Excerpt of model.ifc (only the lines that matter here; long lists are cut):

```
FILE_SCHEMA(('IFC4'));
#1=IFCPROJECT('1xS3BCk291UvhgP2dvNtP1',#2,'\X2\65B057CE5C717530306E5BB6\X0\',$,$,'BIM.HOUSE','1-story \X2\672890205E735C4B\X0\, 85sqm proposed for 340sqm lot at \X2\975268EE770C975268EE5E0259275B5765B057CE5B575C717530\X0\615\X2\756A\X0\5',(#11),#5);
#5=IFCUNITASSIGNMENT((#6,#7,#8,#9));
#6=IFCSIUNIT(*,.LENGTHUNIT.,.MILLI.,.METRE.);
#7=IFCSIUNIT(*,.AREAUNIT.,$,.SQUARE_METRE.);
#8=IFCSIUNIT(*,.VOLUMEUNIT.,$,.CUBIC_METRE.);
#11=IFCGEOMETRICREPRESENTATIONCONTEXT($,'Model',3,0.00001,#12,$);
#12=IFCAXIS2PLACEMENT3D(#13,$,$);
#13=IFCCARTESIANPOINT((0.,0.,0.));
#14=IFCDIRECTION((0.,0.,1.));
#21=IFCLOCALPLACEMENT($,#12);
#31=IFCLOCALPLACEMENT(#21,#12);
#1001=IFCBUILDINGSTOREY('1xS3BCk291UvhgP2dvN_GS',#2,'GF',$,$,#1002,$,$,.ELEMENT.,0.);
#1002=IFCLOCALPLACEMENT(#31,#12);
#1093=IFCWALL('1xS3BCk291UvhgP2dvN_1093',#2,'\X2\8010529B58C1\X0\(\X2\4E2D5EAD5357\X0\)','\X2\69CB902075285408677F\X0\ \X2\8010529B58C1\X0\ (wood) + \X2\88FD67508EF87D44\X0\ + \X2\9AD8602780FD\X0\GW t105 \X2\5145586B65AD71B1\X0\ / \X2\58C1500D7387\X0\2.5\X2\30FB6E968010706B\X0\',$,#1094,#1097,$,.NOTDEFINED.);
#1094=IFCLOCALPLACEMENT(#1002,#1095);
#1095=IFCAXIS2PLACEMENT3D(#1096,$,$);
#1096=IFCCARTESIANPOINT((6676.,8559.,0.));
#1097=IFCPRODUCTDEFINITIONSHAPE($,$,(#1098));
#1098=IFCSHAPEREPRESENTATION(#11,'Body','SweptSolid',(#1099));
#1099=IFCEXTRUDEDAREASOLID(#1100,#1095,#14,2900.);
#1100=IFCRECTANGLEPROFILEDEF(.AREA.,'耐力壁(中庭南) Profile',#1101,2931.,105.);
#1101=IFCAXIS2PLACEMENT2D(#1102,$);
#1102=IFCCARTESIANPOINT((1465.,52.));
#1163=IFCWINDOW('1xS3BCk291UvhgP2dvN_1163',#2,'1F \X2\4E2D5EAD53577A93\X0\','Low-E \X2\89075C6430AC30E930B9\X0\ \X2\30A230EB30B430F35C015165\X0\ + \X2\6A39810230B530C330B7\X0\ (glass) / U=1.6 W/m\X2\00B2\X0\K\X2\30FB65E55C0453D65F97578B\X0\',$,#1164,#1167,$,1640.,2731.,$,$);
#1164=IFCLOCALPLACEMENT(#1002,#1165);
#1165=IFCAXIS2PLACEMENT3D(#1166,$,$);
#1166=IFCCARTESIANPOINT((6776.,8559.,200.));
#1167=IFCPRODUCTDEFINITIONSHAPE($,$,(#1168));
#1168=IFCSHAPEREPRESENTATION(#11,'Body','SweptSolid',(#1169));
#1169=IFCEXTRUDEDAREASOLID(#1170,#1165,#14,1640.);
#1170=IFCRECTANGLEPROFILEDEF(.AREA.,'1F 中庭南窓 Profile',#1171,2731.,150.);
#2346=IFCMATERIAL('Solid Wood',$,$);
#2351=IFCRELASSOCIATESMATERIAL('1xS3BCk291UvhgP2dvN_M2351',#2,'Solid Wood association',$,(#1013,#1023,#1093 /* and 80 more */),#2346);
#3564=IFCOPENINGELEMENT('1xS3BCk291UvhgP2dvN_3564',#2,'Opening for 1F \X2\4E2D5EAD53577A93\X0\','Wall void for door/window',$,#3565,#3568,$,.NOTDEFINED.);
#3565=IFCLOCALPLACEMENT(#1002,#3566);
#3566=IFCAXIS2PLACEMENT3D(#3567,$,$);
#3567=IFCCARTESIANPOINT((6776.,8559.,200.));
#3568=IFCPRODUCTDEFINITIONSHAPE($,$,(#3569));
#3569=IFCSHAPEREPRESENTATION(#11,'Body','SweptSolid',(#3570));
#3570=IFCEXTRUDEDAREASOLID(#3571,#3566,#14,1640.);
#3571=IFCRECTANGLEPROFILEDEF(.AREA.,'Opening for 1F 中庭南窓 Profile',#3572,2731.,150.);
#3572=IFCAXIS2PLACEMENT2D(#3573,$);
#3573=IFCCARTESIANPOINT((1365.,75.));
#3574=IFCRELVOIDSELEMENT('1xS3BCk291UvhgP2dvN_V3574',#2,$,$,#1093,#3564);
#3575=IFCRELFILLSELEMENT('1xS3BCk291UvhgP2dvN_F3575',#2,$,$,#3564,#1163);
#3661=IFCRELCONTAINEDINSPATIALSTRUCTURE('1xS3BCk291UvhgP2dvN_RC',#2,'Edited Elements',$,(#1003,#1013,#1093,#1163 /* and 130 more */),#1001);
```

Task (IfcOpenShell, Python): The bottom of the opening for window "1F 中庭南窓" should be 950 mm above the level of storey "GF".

```python
import numpy as np
import ifcopenshell
import ifcopenshell.api.geometry
import ifcopenshell.geom
import ifcopenshell.util.element
import ifcopenshell.util.placement
import ifcopenshell.util.shape
import ifcopenshell.util.unit

model = ifcopenshell.open("model.ifc")
unit_scale = ifcopenshell.util.unit.calculate_unit_scale(model)

window = model.by_id(1163)
opening = window.FillsVoids[0].RelatingOpeningElement
storey = ifcopenshell.util.element.get_container(window, ifc_class="IfcBuildingStorey")
level = ifcopenshell.util.placement.get_local_placement(storey.ObjectPlacement)[2, 3]

# The opening's origin need not be at the sill, so measure its lowest point.
shape = ifcopenshell.geom.create_shape(ifcopenshell.geom.settings(), opening)
bottom = ifcopenshell.util.shape.get_shape_bottom_elevation(shape, shape.geometry) / unit_scale
dz = level + 0.95 / unit_scale - bottom

shift = np.array([0.0, 0.0, dz])
# The window is not placed relative to its opening, so move both.
for product in (opening, window):
    matrix = ifcopenshell.util.placement.get_local_placement(product.ObjectPlacement)
    matrix[:3, 3] += shift
    ifcopenshell.api.geometry.edit_object_placement(model, product=product, matrix=matrix, is_si=False)

print(f"moved by {dz * unit_scale:+.3f} m")

model.write("model_edited.ifc")
```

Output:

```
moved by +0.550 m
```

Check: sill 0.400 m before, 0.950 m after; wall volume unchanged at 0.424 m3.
